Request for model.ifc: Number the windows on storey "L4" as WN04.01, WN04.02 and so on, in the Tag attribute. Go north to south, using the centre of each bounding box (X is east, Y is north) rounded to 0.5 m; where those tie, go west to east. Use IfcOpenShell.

First a look at what the model holds.

```python
import ifcopenshell
import ifcopenshell.util.element
import ifcopenshell.util.placement

model = ifcopenshell.open("model.ifc")
print(model.schema)
storey = next(s for s in model.by_type("IfcBuildingStorey") if s.Name == "L4")
windows = [e for e in ifcopenshell.util.element.get_decomposition(storey) if e.is_a("IfcWindow")]
for e in sorted(windows, key=lambda e: e.id()):
    origin = ifcopenshell.util.placement.get_local_placement(e.ObjectPlacement)[:3, 3]
    print(e.id(), e.Tag, e.Name, origin.round(2) + 0.0, sep=" | ")
```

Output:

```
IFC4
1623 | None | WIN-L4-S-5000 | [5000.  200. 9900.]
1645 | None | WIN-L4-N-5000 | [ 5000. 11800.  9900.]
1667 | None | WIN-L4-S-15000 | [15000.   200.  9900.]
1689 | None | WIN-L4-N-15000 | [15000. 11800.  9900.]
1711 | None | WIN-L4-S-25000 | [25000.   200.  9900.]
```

```python
import ifcopenshell
import ifcopenshell.geom
import ifcopenshell.util.element
import ifcopenshell.util.shape

model = ifcopenshell.open("model.ifc")
settings = ifcopenshell.geom.settings()
settings.set("use-world-coords", True)


def centre(element):
    shape = ifcopenshell.geom.create_shape(settings, element)
    return ifcopenshell.util.shape.get_bbox_centroid(shape.geometry)


storey = next(s for s in model.by_type("IfcBuildingStorey") if s.Name == "L4")
windows = [e for e in ifcopenshell.util.element.get_decomposition(storey) if e.is_a("IfcWindow")]

# Insertion points can sit at a corner or the storey origin, so sort by the geometry (in metres).
centres = {e: centre(e) for e in windows}
windows.sort(key=lambda e: (-round(centres[e][1] / 0.5), centres[e][0]))

for i, e in enumerate(windows, start=1):
    number = f"WN04.{i:02d}"
    e.Tag = number
    print(e.id(), number)

model.write("model_v2.ifc")
```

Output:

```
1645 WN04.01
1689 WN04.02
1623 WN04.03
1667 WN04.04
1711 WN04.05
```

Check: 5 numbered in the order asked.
